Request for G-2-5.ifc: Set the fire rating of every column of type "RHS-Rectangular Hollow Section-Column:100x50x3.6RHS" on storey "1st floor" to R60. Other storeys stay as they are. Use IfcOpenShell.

First a look at what the model holds.

```python
import ifcopenshell
import ifcopenshell.util.element

model = ifcopenshell.open("G-2-5.ifc")
print(model.schema)
storey = next(s for s in model.by_type("IfcBuildingStorey") if s.Name == "1st floor")
columns = [e for e in ifcopenshell.util.element.get_decomposition(storey) if e.is_a("IfcColumn")]
seen = {}
for e in columns:
    element_type = ifcopenshell.util.element.get_type(e)
    key = (element_type.Name if element_type != e and element_type else None, ifcopenshell.util.element.get_pset(e, "Pset_ColumnCommon", "FireRating"))
    seen[key] = seen.get(key, 0) + 1
for (name, value), count in sorted(seen.items(), key=str):
    print(count, "x", name, "|", value)
```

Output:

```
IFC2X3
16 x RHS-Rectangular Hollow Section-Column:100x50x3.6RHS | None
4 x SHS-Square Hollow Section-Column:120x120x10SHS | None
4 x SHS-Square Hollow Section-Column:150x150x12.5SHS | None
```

```python
import ifcopenshell
import ifcopenshell.api.pset
import ifcopenshell.util.element

model = ifcopenshell.open("G-2-5.ifc")

storey = next(s for s in model.by_type("IfcBuildingStorey") if s.Name == "1st floor")
columns = [e for e in ifcopenshell.util.element.get_decomposition(storey) if e.is_a("IfcColumn")]

count = 0
for e in columns:
    element_type = ifcopenshell.util.element.get_type(e)
    if element_type in (None, e) or element_type.Name != "RHS-Rectangular Hollow Section-Column:100x50x3.6RHS":
        continue
    # add_pset returns the element's existing set when there is one.
    pset = ifcopenshell.api.pset.add_pset(model, product=e, name="Pset_ColumnCommon")
    ifcopenshell.api.pset.edit_pset(model, pset=pset, properties={"FireRating": "R60"})
    count += 1

print(count, "columns updated")

model.write("G-2-5-out.ifc")
```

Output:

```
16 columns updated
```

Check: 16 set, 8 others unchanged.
